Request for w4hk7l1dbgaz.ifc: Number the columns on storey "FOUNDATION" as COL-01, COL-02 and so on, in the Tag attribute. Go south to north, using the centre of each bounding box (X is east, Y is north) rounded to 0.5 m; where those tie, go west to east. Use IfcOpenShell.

First a look at what the model holds.

```python
import ifcopenshell
import ifcopenshell.util.element
import ifcopenshell.util.placement

model = ifcopenshell.open("w4hk7l1dbgaz.ifc")
print(model.schema)
storey = next(s for s in model.by_type("IfcBuildingStorey") if s.Name == "FOUNDATION")
columns = [e for e in ifcopenshell.util.element.get_decomposition(storey) if e.is_a("IfcColumn")]
for e in sorted(columns, key=lambda e: e.id()):
    origin = ifcopenshell.util.placement.get_local_placement(e.ObjectPlacement)[:3, 3]
    print(e.id(), e.Tag, e.Name, origin.round(2) + 0.0, sep=" | ")
```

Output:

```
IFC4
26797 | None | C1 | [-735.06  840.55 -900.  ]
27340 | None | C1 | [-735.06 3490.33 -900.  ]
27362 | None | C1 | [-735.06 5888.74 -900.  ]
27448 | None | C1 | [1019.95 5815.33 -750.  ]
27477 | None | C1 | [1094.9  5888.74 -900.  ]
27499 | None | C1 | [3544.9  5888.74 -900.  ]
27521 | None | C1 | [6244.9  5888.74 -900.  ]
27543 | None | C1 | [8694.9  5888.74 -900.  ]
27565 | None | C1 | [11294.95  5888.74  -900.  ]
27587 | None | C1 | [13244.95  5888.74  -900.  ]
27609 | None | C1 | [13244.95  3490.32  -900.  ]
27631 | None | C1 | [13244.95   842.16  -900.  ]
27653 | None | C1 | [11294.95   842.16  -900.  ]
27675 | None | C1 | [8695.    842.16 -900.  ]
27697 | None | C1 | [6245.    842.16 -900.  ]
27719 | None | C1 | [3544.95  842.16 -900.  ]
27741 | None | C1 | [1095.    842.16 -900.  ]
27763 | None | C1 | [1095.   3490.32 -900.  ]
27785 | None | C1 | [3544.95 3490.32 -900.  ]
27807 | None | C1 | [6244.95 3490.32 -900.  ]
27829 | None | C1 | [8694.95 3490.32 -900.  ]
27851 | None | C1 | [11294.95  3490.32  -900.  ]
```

```python
import ifcopenshell
import ifcopenshell.geom
import ifcopenshell.util.element
import ifcopenshell.util.shape

model = ifcopenshell.open("w4hk7l1dbgaz.ifc")
settings = ifcopenshell.geom.settings()
settings.set("use-world-coords", True)


def centre(element):
    shape = ifcopenshell.geom.create_shape(settings, element)
    return ifcopenshell.util.shape.get_bbox_centroid(shape.geometry)


storey = next(s for s in model.by_type("IfcBuildingStorey") if s.Name == "FOUNDATION")
columns = [e for e in ifcopenshell.util.element.get_decomposition(storey) if e.is_a("IfcColumn")]

# Insertion points can sit at a corner or the storey origin, so sort by the geometry (in metres).
centres = {e: centre(e) for e in columns}
columns.sort(key=lambda e: (round(centres[e][1] / 0.5), centres[e][0]))

for i, e in enumerate(columns, start=1):
    number = f"COL-{i:02d}"
    e.Tag = number
    print(e.id(), number)

model.write("w4hk7l1dbgaz-out.ifc")
```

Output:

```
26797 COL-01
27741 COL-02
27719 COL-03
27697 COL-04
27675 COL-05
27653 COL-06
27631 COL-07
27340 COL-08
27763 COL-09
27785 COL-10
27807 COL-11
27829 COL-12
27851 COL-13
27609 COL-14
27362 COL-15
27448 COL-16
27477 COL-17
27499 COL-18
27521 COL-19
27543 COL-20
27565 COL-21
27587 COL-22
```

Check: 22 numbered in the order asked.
